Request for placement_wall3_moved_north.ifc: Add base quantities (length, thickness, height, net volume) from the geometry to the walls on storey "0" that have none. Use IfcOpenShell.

First a look at what the model holds.

```python
import ifcopenshell
import ifcopenshell.util.element
import ifcopenshell.util.unit

model = ifcopenshell.open("placement_wall3_moved_north.ifc")
print(model.schema)
for unit_type in ("LENGTHUNIT", "AREAUNIT", "VOLUMEUNIT"):
    print(unit_type, ifcopenshell.util.unit.calculate_unit_scale(model, unit_type))
storey = next(s for s in model.by_type("IfcBuildingStorey") if s.Name == "0")
walls = [e for e in ifcopenshell.util.element.get_decomposition(storey) if e.is_a("IfcWall")]
for e in sorted(walls, key=lambda e: e.id()):
    print(e.id(), e.is_a(), e.Name, list(ifcopenshell.util.element.get_psets(e, qtos_only=True)), sep=" | ")
```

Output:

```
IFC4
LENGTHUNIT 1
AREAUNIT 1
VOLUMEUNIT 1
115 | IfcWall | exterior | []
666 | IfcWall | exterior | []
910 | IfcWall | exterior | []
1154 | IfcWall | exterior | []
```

```python
import ifcopenshell
import ifcopenshell.api.pset
import ifcopenshell.geom
import ifcopenshell.util.element
import ifcopenshell.util.shape
import ifcopenshell.util.unit

model = ifcopenshell.open("placement_wall3_moved_north.ifc")
unit_scale = ifcopenshell.util.unit.calculate_unit_scale(model)
volume_scale = ifcopenshell.util.unit.calculate_unit_scale(model, "VOLUMEUNIT")
settings = ifcopenshell.geom.settings()

storey = next(s for s in model.by_type("IfcBuildingStorey") if s.Name == "0")
walls = [e for e in ifcopenshell.util.element.get_decomposition(storey) if e.is_a("IfcWall")]

for e in sorted(walls, key=lambda e: e.id()):
    if ifcopenshell.util.element.get_psets(e, qtos_only=True, should_inherit=False):
        continue
    # Geometry comes back in metres, in the element's own axes.
    shape = ifcopenshell.geom.create_shape(settings, e)
    values = {
        "Length": ifcopenshell.util.shape.get_x(shape.geometry) / unit_scale,
        "Width": ifcopenshell.util.shape.get_y(shape.geometry) / unit_scale,
        "Height": ifcopenshell.util.shape.get_z(shape.geometry) / unit_scale,
        "NetVolume": ifcopenshell.util.shape.get_volume(shape.geometry) / volume_scale,
    }
    qto = ifcopenshell.api.pset.add_qto(model, product=e, name="Qto_WallBaseQuantities")
    ifcopenshell.api.pset.edit_qto(model, qto=qto, properties=values)
    print(e.id(), {k: round(v, 3) for k, v in values.items()})

model.write("placement_wall3_moved_north_updated.ifc")
```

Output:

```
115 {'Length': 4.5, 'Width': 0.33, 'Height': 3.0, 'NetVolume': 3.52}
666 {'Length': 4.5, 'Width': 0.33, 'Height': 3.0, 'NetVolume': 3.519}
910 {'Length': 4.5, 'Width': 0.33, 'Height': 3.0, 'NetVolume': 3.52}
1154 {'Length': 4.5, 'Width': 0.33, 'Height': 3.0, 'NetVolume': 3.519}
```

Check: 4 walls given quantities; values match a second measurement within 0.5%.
